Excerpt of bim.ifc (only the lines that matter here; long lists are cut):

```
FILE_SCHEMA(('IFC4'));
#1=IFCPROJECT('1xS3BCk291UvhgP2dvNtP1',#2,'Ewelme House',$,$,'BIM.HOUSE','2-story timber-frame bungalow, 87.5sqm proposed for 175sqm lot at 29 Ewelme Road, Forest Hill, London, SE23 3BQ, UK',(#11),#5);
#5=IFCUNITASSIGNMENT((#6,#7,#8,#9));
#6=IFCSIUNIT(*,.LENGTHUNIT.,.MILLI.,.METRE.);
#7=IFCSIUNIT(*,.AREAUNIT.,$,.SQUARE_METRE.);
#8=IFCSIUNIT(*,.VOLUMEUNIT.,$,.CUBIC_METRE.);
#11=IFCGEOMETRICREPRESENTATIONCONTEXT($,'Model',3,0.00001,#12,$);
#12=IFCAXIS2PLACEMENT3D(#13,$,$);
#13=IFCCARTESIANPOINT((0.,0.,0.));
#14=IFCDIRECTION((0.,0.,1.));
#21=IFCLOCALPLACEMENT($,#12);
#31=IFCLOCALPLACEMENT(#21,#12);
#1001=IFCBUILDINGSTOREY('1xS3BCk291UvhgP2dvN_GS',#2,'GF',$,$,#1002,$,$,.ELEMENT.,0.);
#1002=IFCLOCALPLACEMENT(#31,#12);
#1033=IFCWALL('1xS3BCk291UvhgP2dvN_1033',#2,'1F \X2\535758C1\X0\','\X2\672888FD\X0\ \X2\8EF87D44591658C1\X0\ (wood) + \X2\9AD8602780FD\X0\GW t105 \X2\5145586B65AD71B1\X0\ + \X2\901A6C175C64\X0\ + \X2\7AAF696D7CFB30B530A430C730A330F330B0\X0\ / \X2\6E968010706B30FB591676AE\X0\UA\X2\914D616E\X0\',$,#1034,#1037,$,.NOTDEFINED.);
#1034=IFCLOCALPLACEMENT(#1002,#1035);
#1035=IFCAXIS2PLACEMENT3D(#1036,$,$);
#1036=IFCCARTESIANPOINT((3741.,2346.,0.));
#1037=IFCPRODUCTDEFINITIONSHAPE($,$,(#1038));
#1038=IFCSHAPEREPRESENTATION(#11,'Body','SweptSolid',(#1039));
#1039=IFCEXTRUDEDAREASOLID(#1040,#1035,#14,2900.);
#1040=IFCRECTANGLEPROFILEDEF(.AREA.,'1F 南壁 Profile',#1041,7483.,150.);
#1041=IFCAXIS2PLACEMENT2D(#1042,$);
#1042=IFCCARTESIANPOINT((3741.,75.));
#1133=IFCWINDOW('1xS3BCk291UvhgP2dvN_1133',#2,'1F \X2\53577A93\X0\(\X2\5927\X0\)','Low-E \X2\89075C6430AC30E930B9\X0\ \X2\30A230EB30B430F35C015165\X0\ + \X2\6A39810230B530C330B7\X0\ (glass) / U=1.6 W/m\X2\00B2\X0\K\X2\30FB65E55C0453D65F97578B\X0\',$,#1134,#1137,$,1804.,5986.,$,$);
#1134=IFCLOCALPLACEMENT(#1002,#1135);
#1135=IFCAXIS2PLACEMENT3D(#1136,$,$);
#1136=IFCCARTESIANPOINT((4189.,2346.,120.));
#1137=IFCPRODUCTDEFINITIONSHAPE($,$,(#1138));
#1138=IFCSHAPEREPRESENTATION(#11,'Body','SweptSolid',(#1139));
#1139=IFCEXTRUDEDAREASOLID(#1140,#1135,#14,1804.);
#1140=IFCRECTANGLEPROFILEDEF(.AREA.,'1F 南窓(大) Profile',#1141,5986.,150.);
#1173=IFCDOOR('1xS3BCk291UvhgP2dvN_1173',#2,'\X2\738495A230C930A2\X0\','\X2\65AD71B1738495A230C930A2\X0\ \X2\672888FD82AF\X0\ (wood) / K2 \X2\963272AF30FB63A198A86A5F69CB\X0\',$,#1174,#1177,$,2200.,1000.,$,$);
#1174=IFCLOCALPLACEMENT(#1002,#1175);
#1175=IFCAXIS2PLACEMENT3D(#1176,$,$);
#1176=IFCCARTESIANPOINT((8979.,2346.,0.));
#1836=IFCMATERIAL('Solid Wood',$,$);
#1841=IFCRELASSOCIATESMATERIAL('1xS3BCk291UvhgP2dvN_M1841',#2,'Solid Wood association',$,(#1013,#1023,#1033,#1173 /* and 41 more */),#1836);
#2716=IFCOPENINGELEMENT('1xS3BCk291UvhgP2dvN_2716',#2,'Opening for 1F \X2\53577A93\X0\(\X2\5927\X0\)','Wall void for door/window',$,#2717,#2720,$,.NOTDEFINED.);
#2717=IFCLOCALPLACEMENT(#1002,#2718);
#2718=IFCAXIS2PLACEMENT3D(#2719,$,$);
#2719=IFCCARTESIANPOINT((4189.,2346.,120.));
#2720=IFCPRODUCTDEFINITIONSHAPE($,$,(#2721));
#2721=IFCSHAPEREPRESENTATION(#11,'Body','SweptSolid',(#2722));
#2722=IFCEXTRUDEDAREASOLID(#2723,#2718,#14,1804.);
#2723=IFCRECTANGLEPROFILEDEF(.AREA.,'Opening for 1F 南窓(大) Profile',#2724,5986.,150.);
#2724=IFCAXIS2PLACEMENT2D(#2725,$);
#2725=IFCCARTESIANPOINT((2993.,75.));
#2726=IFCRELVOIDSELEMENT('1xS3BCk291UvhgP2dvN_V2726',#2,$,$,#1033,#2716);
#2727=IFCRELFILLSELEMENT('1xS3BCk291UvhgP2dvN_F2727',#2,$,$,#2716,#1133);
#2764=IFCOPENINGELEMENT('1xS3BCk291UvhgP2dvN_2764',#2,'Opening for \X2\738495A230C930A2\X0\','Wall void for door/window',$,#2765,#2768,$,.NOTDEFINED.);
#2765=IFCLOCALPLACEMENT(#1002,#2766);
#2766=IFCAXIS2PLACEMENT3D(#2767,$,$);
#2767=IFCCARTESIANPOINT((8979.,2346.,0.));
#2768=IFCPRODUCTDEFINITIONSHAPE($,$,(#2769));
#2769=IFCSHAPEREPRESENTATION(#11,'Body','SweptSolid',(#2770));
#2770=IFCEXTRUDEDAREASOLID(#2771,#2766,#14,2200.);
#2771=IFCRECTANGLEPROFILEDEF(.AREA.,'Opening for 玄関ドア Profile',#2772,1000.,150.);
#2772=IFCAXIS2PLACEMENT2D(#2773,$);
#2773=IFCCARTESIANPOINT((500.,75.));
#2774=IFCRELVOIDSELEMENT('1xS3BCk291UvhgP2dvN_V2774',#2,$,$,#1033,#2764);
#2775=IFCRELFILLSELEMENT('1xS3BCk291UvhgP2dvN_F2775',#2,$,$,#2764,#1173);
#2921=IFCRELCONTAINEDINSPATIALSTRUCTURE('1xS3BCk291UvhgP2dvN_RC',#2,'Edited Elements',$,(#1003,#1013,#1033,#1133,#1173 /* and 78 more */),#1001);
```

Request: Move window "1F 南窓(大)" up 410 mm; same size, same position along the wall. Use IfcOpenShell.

```python
import numpy as np
import ifcopenshell
import ifcopenshell.api.geometry
import ifcopenshell.util.placement
import ifcopenshell.util.unit

model = ifcopenshell.open("bim.ifc")
unit_scale = ifcopenshell.util.unit.calculate_unit_scale(model)

window = model.by_guid("1xS3BCk291UvhgP2dvN_1133")
opening = window.FillsVoids[0].RelatingOpeningElement
dz = 0.41 / unit_scale

shift = np.array([0.0, 0.0, dz])
# The window is not placed relative to its opening, so move both.
for product in (opening, window):
    matrix = ifcopenshell.util.placement.get_local_placement(product.ObjectPlacement)
    matrix[:3, 3] += shift
    ifcopenshell.api.geometry.edit_object_placement(model, product=product, matrix=matrix, is_si=False)

print(f"moved by {dz * unit_scale:+.3f} m")

model.write("bim_edited.ifc")
```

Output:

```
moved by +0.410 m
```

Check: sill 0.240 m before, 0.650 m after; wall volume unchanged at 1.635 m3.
